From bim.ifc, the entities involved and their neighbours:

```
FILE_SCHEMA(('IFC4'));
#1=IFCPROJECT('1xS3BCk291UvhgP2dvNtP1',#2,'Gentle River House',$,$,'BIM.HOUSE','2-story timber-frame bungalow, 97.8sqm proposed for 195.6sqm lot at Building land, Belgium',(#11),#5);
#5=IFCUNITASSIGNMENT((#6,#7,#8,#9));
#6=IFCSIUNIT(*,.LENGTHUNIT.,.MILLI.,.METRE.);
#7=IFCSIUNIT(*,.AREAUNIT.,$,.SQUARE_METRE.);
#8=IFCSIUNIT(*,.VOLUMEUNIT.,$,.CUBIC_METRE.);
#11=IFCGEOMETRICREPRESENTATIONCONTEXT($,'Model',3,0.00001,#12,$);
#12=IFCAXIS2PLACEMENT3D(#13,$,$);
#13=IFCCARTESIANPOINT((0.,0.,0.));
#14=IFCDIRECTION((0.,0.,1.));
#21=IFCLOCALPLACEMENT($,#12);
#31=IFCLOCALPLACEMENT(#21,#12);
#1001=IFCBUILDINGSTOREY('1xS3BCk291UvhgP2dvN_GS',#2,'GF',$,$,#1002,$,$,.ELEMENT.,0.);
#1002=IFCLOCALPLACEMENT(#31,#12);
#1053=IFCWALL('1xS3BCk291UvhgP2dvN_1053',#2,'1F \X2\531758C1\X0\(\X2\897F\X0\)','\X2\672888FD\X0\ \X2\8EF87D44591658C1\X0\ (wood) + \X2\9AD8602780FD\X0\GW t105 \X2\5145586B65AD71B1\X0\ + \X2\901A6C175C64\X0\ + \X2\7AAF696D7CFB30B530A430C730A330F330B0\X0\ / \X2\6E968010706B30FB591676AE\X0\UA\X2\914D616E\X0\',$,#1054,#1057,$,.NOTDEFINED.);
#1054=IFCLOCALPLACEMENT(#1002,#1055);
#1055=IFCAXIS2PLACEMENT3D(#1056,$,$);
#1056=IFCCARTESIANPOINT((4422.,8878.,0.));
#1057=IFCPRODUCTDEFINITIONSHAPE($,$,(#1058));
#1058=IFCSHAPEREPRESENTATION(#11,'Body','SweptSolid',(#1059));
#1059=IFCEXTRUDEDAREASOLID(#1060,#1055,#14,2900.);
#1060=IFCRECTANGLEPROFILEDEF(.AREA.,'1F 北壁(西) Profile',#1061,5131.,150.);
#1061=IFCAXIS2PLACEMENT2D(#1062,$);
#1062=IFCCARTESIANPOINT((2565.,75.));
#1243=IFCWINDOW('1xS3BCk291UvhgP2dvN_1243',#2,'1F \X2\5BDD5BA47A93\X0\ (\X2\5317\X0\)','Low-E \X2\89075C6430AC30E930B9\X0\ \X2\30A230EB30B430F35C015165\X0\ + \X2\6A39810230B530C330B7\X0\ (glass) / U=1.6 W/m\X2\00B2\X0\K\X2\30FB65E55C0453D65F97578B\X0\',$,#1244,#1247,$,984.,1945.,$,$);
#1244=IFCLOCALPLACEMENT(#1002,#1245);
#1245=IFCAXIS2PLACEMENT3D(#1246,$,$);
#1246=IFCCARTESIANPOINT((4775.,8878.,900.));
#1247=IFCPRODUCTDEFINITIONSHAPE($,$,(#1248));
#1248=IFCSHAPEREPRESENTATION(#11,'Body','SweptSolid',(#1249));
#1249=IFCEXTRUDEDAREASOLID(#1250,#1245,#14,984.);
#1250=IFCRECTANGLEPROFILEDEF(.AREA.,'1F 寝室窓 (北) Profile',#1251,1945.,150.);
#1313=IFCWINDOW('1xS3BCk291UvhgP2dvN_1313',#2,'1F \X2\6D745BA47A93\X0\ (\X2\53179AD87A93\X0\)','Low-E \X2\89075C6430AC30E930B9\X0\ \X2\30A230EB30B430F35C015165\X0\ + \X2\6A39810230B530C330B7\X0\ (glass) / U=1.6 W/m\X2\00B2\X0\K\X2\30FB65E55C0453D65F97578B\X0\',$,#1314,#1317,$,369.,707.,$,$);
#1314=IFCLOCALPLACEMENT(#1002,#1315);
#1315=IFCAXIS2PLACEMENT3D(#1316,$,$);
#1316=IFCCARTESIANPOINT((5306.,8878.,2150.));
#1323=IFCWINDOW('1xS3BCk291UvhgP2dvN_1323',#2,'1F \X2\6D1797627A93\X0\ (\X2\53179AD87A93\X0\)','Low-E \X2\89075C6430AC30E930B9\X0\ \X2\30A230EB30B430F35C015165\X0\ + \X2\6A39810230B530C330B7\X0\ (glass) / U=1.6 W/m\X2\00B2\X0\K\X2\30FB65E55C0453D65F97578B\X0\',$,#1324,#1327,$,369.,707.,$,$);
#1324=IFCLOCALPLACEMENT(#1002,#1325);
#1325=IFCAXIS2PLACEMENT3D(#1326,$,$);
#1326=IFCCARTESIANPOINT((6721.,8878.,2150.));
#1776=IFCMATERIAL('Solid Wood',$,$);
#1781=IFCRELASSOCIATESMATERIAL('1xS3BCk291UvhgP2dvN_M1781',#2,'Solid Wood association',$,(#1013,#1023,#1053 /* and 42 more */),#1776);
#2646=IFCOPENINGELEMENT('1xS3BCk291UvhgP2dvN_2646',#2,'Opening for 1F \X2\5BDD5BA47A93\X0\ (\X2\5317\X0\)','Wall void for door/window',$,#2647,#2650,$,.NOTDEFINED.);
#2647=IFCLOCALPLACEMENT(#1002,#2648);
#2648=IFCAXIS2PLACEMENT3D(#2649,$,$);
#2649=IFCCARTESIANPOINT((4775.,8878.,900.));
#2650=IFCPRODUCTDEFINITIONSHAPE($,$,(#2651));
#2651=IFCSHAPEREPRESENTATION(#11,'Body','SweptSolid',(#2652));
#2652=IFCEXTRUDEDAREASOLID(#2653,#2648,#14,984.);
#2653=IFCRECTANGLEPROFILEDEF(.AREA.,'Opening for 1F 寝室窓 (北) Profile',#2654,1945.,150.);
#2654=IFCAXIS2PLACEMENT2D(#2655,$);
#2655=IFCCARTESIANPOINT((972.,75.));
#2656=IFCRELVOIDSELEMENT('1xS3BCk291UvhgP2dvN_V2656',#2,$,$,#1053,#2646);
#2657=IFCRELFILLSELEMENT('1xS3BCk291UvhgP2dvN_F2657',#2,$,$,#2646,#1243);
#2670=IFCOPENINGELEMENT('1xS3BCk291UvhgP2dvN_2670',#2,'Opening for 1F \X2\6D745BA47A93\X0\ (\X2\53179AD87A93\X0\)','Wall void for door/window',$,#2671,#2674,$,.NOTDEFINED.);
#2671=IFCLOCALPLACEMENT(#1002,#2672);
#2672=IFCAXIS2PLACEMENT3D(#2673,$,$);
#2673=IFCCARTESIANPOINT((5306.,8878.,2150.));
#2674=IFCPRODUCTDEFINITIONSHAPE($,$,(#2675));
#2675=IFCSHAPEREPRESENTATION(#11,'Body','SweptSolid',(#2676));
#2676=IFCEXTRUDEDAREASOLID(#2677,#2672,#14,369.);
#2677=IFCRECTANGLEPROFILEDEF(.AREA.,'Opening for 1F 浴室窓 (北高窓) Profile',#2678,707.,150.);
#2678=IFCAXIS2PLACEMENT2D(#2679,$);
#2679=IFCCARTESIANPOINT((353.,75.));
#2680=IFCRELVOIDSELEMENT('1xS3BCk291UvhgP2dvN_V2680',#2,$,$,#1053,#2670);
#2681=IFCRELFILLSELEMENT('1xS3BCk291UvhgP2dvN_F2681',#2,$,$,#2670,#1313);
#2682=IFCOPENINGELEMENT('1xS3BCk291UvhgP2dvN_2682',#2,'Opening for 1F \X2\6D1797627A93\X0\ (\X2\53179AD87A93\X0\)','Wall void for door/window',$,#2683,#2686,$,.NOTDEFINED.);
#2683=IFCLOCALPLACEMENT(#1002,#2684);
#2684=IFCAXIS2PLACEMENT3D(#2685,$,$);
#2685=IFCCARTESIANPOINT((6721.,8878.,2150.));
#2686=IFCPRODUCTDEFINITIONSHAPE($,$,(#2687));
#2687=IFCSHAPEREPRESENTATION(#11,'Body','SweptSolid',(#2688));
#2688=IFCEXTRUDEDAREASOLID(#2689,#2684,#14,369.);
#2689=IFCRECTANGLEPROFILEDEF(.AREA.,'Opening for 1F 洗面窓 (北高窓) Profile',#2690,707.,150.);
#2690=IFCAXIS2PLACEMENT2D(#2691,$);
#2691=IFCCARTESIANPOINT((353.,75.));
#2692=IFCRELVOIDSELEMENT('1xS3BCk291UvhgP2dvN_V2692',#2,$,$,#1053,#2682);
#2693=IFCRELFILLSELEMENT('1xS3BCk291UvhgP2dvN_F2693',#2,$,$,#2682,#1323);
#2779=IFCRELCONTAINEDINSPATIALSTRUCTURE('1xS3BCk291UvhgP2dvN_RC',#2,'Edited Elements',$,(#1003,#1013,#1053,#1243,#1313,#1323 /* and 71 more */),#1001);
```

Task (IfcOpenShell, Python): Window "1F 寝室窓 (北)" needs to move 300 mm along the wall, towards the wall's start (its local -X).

```python
import ifcopenshell
import ifcopenshell.api.geometry
import ifcopenshell.util.placement
import ifcopenshell.util.unit

model = ifcopenshell.open("bim.ifc")
unit_scale = ifcopenshell.util.unit.calculate_unit_scale(model)

window = model.by_guid("1xS3BCk291UvhgP2dvN_1243")
opening = window.FillsVoids[0].RelatingOpeningElement
wall = opening.VoidsElements[0].RelatingBuildingElement

wall_matrix = ifcopenshell.util.placement.get_local_placement(wall.ObjectPlacement)
shift = wall_matrix[:3, 0] * -0.3 / unit_scale
before = ifcopenshell.util.placement.get_local_placement(window.ObjectPlacement)[:3, 3].copy()

# The window is not placed relative to its opening, so move both.
for product in (opening, window):
    matrix = ifcopenshell.util.placement.get_local_placement(product.ObjectPlacement)
    matrix[:3, 3] += shift
    ifcopenshell.api.geometry.edit_object_placement(model, product=product, matrix=matrix, is_si=False)

after = ifcopenshell.util.placement.get_local_placement(window.ObjectPlacement)[:3, 3]
print("window moved by", (after - before).round(3) + 0.0)

model.write("bim_updated.ifc")
```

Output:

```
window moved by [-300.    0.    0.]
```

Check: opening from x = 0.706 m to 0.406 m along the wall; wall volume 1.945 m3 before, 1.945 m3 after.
